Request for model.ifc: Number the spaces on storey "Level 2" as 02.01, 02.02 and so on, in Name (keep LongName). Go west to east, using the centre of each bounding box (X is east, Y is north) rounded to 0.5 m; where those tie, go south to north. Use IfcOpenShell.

First a look at what the model holds.

```python
import ifcopenshell
import ifcopenshell.util.element
import ifcopenshell.util.placement

model = ifcopenshell.open("model.ifc")
print(model.schema)
storey = next(s for s in model.by_type("IfcBuildingStorey") if s.Name == "Level 2")
spaces = [e for e in ifcopenshell.util.element.get_decomposition(storey) if e.is_a("IfcSpace")]
for e in sorted(spaces, key=lambda e: e.id()):
    origin = ifcopenshell.util.placement.get_local_placement(e.ObjectPlacement)[:3, 3]
    print(e.id(), e.Name, e.LongName, origin.round(2) + 0.0, sep=" | ")
```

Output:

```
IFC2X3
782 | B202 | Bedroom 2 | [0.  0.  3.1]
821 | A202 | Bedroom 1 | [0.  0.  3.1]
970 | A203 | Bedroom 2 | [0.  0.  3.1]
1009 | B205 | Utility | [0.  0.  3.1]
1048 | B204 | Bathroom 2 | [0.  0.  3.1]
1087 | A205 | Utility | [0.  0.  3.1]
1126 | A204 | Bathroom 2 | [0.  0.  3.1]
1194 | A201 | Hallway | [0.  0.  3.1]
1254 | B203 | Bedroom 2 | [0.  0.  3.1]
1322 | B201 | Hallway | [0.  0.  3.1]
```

```python
import ifcopenshell
import ifcopenshell.geom
import ifcopenshell.util.element
import ifcopenshell.util.shape

model = ifcopenshell.open("model.ifc")
settings = ifcopenshell.geom.settings()
settings.set("use-world-coords", True)


def centre(element):
    shape = ifcopenshell.geom.create_shape(settings, element)
    return ifcopenshell.util.shape.get_bbox_centroid(shape.geometry)


storey = next(s for s in model.by_type("IfcBuildingStorey") if s.Name == "Level 2")
spaces = [e for e in ifcopenshell.util.element.get_decomposition(storey) if e.is_a("IfcSpace")]

# Insertion points can sit at a corner or the storey origin, so sort by the geometry (in metres).
centres = {e: centre(e) for e in spaces}
spaces.sort(key=lambda e: (round(centres[e][0] / 0.5), centres[e][1]))

for i, e in enumerate(spaces, start=1):
    number = f"02.{i:02d}"
    e.Name = number
    print(e.id(), number)

model.write("model_edited.ifc")
```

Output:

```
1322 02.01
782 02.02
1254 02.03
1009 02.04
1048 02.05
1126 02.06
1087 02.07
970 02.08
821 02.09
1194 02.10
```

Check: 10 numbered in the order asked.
